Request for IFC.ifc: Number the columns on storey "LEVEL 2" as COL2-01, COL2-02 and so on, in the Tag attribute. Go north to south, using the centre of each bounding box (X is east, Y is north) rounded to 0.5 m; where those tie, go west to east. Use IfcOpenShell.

First a look at what the model holds.

```python
import ifcopenshell
import ifcopenshell.util.element
import ifcopenshell.util.placement

model = ifcopenshell.open("IFC.ifc")
print(model.schema)
storey = next(s for s in model.by_type("IfcBuildingStorey") if s.Name == "LEVEL 2")
columns = [e for e in ifcopenshell.util.element.get_decomposition(storey) if e.is_a("IfcColumn")]
for e in sorted(columns, key=lambda e: e.id()):
    origin = ifcopenshell.util.placement.get_local_placement(e.ObjectPlacement)[:3, 3]
    print(e.id(), e.Tag, e.Name, origin.round(2) + 0.0, sep=" | ")
```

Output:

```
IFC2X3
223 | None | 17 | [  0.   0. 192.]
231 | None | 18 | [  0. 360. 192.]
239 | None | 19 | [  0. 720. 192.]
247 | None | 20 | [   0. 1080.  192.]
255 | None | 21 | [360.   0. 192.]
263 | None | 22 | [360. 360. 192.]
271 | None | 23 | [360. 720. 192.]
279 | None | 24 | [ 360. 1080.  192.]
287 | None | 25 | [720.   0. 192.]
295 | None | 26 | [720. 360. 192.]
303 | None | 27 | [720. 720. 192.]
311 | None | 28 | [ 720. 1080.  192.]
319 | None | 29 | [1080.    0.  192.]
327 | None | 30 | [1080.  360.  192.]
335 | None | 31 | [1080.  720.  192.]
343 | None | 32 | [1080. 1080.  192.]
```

```python
import ifcopenshell
import ifcopenshell.geom
import ifcopenshell.util.element
import ifcopenshell.util.shape

model = ifcopenshell.open("IFC.ifc")
settings = ifcopenshell.geom.settings()
settings.set("use-world-coords", True)


def centre(element):
    shape = ifcopenshell.geom.create_shape(settings, element)
    return ifcopenshell.util.shape.get_bbox_centroid(shape.geometry)


storey = next(s for s in model.by_type("IfcBuildingStorey") if s.Name == "LEVEL 2")
columns = [e for e in ifcopenshell.util.element.get_decomposition(storey) if e.is_a("IfcColumn")]

# Insertion points can sit at a corner or the storey origin, so sort by the geometry (in metres).
centres = {e: centre(e) for e in columns}
columns.sort(key=lambda e: (-round(centres[e][1] / 0.5), centres[e][0]))

for i, e in enumerate(columns, start=1):
    number = f"COL2-{i:02d}"
    e.Tag = number
    print(e.id(), number)

model.write("IFC_rev.ifc")
```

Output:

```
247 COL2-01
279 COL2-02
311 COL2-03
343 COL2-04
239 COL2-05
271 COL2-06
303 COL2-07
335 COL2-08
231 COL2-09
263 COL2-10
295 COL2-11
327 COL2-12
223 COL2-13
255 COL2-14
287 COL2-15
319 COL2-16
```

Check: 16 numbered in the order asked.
